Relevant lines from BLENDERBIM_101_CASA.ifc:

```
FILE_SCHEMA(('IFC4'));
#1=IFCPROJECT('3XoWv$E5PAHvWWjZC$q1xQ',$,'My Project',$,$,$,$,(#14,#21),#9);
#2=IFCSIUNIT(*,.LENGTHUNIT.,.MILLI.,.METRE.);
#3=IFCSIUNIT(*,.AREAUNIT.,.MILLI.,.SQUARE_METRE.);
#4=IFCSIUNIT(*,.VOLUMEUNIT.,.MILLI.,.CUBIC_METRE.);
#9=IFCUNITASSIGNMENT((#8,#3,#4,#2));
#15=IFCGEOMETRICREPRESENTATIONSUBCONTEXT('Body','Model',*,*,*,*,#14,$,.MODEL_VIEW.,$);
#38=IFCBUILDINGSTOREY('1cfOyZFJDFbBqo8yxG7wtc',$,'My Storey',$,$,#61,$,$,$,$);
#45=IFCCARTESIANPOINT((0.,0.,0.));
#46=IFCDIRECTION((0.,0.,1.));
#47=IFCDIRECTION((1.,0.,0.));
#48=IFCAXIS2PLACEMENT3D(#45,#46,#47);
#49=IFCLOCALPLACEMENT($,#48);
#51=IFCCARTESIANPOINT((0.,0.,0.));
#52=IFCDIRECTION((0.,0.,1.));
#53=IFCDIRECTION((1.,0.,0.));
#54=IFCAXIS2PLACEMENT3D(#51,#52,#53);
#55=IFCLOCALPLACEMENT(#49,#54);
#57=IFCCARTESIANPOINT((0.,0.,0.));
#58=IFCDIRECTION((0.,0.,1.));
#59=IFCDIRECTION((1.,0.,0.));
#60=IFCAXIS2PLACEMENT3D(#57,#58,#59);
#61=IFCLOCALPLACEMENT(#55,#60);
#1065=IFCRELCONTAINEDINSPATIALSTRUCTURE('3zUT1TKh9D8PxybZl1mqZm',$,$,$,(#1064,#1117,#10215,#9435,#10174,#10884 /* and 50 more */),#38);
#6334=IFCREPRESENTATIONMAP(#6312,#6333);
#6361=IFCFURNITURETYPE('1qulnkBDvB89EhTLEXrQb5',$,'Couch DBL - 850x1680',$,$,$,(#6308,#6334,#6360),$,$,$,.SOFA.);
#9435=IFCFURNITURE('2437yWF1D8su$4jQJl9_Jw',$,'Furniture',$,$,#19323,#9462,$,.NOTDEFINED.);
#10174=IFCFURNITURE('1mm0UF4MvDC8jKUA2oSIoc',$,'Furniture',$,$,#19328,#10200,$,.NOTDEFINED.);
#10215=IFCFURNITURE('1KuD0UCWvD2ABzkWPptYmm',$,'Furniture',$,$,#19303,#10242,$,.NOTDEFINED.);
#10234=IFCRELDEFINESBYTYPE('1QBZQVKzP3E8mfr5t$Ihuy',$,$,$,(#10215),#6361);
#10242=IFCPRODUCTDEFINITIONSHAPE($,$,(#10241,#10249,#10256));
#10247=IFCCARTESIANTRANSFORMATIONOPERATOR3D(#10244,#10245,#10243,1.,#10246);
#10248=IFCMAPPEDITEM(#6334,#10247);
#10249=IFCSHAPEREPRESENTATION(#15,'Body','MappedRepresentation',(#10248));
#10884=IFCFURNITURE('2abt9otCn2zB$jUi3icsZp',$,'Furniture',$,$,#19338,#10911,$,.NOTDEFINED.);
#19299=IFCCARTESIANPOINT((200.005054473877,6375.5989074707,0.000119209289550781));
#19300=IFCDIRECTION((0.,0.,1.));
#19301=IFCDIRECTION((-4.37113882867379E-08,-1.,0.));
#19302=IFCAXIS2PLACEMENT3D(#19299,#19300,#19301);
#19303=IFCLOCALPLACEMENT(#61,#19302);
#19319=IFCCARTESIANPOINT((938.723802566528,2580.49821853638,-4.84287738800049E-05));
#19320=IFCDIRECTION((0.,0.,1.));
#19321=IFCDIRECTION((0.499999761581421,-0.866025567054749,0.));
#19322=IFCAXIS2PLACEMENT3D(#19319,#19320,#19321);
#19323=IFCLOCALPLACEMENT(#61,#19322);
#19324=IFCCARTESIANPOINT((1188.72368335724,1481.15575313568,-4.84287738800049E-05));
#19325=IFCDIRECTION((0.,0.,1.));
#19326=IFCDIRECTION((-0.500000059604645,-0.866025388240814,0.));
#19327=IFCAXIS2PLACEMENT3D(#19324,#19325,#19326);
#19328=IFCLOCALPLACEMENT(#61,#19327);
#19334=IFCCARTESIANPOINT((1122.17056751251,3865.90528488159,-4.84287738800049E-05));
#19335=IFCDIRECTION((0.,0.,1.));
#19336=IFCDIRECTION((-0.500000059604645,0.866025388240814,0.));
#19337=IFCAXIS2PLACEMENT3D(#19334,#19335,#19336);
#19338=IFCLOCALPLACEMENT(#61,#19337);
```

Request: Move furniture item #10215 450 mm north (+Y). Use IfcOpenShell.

```python
import ifcopenshell
import ifcopenshell.api.geometry
import ifcopenshell.util.placement
import ifcopenshell.util.unit

model = ifcopenshell.open("BLENDERBIM_101_CASA.ifc")
unit_scale = ifcopenshell.util.unit.calculate_unit_scale(model)

item = model.by_id(10215)
matrix = ifcopenshell.util.placement.get_local_placement(item.ObjectPlacement)
matrix[1, 3] += 0.45 / unit_scale
ifcopenshell.api.geometry.edit_object_placement(model, product=item, matrix=matrix, is_si=False)

print(ifcopenshell.util.placement.get_local_placement(item.ObjectPlacement).round(3) + 0.0)

model.write("BLENDERBIM_101_CASA_edited.ifc")
```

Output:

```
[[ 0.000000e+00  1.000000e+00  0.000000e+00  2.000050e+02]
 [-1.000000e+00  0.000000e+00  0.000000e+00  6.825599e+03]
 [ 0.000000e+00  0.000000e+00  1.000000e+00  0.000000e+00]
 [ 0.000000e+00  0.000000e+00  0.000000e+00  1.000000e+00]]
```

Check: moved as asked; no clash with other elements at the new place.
